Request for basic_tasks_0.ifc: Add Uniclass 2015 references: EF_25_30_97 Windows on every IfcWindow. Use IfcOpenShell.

First a look at what the model holds.

```python
import ifcopenshell

model = ifcopenshell.open("basic_tasks_0.ifc")
print(model.schema)
print("classifications:", [c.Name for c in model.by_type("IfcClassification")])
for ifc_class in ("IfcDoor", "IfcRoof", "IfcStair", "IfcWall", "IfcWindow"):
    print(ifc_class, len(model.by_type(ifc_class)))
```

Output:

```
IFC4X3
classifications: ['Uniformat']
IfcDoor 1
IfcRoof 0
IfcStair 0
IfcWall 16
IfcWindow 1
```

```python
import ifcopenshell
import ifcopenshell.api.classification

model = ifcopenshell.open("basic_tasks_0.ifc")

system = ifcopenshell.api.classification.add_classification(model, classification="Uniclass 2015")

codes = {
    "IfcWindow": ("EF_25_30_97", "Windows"),
}
for ifc_class, (code, name) in codes.items():
    products = model.by_type(ifc_class)
    ifcopenshell.api.classification.add_reference(
        model, products=products, classification=system, identification=code, name=name
    )
    print(code, len(products))

model.write("basic_tasks_0_rev.ifc")
```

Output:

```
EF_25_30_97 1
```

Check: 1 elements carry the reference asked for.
